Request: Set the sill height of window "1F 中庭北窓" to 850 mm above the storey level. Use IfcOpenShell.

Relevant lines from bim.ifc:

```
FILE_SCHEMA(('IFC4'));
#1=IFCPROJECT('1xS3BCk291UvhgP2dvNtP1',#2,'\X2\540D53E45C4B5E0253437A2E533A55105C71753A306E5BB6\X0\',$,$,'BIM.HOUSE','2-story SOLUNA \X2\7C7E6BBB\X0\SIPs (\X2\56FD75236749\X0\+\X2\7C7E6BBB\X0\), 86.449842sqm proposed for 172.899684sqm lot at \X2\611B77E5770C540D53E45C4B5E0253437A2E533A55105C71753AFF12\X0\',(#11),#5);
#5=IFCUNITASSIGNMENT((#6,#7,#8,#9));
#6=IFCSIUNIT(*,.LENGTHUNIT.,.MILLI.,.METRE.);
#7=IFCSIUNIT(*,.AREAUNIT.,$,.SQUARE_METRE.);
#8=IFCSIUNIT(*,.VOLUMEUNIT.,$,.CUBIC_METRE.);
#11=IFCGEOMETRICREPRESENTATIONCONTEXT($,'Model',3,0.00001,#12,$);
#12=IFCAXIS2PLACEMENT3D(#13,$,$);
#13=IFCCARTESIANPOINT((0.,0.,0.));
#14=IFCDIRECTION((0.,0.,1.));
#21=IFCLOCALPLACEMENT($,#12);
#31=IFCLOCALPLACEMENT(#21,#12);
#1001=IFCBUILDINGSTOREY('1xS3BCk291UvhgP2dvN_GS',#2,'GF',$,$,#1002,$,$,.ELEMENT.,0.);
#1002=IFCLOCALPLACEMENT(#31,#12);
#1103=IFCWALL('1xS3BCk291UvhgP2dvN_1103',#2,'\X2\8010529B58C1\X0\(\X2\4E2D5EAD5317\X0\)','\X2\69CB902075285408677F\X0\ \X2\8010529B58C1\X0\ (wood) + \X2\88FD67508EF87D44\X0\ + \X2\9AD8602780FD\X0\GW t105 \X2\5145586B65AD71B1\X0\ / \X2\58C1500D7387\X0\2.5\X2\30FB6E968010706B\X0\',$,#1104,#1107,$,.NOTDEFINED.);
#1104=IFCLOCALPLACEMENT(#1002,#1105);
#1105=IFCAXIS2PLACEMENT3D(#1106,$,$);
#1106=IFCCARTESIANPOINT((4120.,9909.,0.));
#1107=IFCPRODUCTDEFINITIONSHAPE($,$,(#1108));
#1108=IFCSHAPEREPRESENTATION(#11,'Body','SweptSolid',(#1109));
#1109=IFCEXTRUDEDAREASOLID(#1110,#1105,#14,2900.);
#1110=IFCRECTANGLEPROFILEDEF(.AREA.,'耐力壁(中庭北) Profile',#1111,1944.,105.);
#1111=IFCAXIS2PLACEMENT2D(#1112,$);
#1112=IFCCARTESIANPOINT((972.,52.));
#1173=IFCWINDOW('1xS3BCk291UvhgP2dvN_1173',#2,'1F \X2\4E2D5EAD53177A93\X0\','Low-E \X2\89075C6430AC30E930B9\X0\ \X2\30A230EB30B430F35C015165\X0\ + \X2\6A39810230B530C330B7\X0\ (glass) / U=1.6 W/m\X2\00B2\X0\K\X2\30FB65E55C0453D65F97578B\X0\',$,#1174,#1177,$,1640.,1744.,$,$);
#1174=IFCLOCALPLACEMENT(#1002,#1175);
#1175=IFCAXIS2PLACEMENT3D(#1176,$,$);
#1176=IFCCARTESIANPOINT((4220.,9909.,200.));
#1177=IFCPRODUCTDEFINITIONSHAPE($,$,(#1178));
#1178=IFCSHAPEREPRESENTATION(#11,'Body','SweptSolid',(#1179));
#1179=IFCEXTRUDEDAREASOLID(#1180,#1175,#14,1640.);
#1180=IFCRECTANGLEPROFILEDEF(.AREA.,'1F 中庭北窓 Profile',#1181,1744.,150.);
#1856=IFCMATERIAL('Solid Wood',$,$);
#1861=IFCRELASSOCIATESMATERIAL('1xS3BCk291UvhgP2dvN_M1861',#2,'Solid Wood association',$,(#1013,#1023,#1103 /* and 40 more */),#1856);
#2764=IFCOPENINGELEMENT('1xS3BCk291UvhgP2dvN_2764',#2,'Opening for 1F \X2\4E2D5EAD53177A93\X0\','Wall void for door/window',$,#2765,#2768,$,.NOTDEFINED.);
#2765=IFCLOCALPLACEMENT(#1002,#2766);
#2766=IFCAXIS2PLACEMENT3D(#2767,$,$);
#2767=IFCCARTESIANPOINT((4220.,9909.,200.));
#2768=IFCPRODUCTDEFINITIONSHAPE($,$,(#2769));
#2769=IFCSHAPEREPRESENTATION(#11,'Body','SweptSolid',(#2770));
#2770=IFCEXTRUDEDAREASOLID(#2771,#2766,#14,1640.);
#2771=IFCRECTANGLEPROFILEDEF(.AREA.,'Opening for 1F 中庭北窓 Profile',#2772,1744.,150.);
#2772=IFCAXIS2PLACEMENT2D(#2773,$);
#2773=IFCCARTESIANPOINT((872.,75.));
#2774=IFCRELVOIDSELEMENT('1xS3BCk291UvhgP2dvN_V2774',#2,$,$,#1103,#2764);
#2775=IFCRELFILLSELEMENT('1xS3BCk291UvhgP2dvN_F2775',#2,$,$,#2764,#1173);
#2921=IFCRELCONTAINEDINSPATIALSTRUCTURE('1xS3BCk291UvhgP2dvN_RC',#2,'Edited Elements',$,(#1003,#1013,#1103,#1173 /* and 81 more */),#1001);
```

```python
import numpy as np
import ifcopenshell
import ifcopenshell.api.geometry
import ifcopenshell.geom
import ifcopenshell.util.element
import ifcopenshell.util.placement
import ifcopenshell.util.shape
import ifcopenshell.util.unit

model = ifcopenshell.open("bim.ifc")
unit_scale = ifcopenshell.util.unit.calculate_unit_scale(model)

window = model.by_guid("1xS3BCk291UvhgP2dvN_1173")
opening = window.FillsVoids[0].RelatingOpeningElement
storey = ifcopenshell.util.element.get_container(window, ifc_class="IfcBuildingStorey")
level = ifcopenshell.util.placement.get_local_placement(storey.ObjectPlacement)[2, 3]

# The opening's origin need not be at the sill, so measure its lowest point.
shape = ifcopenshell.geom.create_shape(ifcopenshell.geom.settings(), opening)
bottom = ifcopenshell.util.shape.get_shape_bottom_elevation(shape, shape.geometry) / unit_scale
dz = level + 850.0 - bottom

shift = np.array([0.0, 0.0, dz])
# The window is not placed relative to its opening, so move both.
for product in (opening, window):
    matrix = ifcopenshell.util.placement.get_local_placement(product.ObjectPlacement)
    matrix[:3, 3] += shift
    ifcopenshell.api.geometry.edit_object_placement(model, product=product, matrix=matrix, is_si=False)

print(f"moved by {dz * unit_scale:+.3f} m")

model.write("bim_v2.ifc")
```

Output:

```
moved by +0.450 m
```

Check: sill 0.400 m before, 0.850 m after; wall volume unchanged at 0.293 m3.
